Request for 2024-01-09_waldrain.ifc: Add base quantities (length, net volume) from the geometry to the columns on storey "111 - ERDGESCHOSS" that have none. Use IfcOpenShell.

First a look at what the model holds.

```python
import ifcopenshell
import ifcopenshell.util.element
import ifcopenshell.util.unit

model = ifcopenshell.open("2024-01-09_waldrain.ifc")
print(model.schema)
for unit_type in ("LENGTHUNIT", "AREAUNIT", "VOLUMEUNIT"):
    print(unit_type, ifcopenshell.util.unit.calculate_unit_scale(model, unit_type))
storey = next(s for s in model.by_type("IfcBuildingStorey") if s.Name == "111 - ERDGESCHOSS")
columns = [e for e in ifcopenshell.util.element.get_decomposition(storey) if e.is_a("IfcColumn")]
for e in sorted(columns, key=lambda e: e.id()):
    print(e.id(), e.is_a(), e.Name, list(ifcopenshell.util.element.get_psets(e, qtos_only=True)), sep=" | ")
```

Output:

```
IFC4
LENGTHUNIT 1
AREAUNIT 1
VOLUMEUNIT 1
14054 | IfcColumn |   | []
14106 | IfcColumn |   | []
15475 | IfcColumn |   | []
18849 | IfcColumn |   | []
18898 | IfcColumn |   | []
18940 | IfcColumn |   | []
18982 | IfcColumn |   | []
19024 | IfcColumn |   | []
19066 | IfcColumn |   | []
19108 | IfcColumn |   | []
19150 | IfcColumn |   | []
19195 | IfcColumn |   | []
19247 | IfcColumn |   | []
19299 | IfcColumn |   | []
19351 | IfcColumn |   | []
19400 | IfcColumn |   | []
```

```python
import ifcopenshell
import ifcopenshell.api.pset
import ifcopenshell.geom
import ifcopenshell.util.element
import ifcopenshell.util.shape
import ifcopenshell.util.unit

model = ifcopenshell.open("2024-01-09_waldrain.ifc")
unit_scale = ifcopenshell.util.unit.calculate_unit_scale(model)
volume_scale = ifcopenshell.util.unit.calculate_unit_scale(model, "VOLUMEUNIT")
settings = ifcopenshell.geom.settings()

storey = next(s for s in model.by_type("IfcBuildingStorey") if s.Name == "111 - ERDGESCHOSS")
columns = [e for e in ifcopenshell.util.element.get_decomposition(storey) if e.is_a("IfcColumn")]

for e in sorted(columns, key=lambda e: e.id()):
    if ifcopenshell.util.element.get_psets(e, qtos_only=True, should_inherit=False):
        continue
    # Geometry comes back in metres, in the element's own axes.
    shape = ifcopenshell.geom.create_shape(settings, e)
    values = {
        "Length": ifcopenshell.util.shape.get_z(shape.geometry) / unit_scale,
        "NetVolume": ifcopenshell.util.shape.get_volume(shape.geometry) / volume_scale,
    }
    qto = ifcopenshell.api.pset.add_qto(model, product=e, name="Qto_ColumnBaseQuantities")
    ifcopenshell.api.pset.edit_qto(model, qto=qto, properties=values)
    print(e.id(), {k: round(v, 3) for k, v in values.items()})

model.write("2024-01-09_waldrain-out.ifc")
```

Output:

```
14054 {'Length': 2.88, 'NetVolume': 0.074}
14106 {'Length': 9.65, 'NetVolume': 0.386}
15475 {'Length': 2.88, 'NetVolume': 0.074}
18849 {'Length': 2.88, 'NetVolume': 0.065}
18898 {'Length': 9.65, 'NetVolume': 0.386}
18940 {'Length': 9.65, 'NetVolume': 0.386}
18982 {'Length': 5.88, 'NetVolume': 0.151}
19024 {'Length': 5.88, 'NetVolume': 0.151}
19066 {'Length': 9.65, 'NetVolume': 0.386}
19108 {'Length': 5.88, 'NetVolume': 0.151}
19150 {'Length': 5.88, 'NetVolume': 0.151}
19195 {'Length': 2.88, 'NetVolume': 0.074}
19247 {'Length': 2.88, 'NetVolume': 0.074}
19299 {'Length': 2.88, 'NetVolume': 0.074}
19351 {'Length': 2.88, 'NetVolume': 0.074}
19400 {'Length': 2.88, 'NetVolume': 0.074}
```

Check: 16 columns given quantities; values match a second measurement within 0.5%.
